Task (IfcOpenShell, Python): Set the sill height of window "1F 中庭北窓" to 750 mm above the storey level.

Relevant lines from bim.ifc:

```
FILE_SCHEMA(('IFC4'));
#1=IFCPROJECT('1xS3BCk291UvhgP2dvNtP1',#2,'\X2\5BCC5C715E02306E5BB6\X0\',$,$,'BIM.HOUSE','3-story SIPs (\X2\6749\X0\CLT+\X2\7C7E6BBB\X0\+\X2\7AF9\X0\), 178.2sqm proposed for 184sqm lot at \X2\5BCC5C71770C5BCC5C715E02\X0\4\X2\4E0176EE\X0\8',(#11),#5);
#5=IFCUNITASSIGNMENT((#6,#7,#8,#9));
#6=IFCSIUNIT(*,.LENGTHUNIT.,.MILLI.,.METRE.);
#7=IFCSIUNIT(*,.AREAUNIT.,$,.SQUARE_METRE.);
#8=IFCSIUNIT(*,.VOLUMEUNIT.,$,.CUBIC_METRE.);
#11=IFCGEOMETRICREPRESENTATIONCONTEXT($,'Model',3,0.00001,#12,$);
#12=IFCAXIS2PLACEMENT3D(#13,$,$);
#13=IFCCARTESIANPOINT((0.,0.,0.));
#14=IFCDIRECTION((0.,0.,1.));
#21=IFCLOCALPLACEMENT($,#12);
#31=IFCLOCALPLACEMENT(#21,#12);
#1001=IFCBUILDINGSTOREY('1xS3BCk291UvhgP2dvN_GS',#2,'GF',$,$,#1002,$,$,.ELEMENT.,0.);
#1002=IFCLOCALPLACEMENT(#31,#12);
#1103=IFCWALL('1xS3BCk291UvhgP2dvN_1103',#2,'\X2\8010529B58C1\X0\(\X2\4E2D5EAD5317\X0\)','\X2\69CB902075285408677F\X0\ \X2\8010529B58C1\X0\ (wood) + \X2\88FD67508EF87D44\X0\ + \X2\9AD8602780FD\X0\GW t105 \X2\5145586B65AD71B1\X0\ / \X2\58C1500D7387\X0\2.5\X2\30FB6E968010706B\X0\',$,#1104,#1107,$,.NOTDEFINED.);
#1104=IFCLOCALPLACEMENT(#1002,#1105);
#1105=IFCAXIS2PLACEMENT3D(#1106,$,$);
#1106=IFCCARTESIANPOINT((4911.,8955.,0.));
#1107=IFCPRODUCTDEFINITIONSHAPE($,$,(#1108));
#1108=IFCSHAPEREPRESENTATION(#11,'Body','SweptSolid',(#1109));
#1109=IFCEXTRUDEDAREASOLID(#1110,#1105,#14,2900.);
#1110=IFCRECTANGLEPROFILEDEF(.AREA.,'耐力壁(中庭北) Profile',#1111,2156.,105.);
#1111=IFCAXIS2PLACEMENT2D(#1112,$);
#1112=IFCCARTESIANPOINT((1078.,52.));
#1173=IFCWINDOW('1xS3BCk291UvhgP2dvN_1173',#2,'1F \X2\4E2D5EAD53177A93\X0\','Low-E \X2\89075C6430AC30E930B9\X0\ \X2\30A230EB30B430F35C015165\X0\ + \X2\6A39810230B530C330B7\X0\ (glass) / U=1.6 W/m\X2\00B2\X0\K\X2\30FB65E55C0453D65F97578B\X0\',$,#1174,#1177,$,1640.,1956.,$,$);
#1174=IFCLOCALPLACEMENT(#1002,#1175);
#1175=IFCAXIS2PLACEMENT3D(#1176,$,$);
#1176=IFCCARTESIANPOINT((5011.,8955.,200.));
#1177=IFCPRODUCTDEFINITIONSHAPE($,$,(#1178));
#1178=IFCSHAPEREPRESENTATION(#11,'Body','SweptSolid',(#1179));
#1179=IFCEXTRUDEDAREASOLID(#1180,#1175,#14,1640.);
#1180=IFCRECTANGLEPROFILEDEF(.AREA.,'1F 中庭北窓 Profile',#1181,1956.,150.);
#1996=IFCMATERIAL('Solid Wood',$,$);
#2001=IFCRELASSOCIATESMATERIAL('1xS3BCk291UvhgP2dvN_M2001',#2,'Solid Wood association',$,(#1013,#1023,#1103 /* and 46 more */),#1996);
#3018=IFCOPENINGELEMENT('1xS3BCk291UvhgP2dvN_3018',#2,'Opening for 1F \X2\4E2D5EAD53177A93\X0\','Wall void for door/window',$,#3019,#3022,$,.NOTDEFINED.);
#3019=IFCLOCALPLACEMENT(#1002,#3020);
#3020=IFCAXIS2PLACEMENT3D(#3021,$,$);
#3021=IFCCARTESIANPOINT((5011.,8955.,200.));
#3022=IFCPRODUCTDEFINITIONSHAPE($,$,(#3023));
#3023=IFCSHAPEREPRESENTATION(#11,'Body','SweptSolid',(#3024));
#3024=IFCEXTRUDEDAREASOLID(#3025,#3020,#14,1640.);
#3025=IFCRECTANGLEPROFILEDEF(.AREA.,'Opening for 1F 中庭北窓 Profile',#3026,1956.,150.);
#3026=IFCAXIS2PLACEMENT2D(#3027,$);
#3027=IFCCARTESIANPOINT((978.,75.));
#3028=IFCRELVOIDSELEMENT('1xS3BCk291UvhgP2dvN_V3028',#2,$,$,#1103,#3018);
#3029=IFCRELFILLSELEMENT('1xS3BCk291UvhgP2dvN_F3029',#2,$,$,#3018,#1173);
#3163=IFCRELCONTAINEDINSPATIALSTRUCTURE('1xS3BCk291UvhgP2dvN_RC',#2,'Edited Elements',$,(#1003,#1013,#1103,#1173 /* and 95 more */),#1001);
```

```python
import numpy as np
import ifcopenshell
import ifcopenshell.api.geometry
import ifcopenshell.geom
import ifcopenshell.util.element
import ifcopenshell.util.placement
import ifcopenshell.util.shape
import ifcopenshell.util.unit

model = ifcopenshell.open("bim.ifc")
unit_scale = ifcopenshell.util.unit.calculate_unit_scale(model)

window = model.by_guid("1xS3BCk291UvhgP2dvN_1173")
opening = window.FillsVoids[0].RelatingOpeningElement
storey = ifcopenshell.util.element.get_container(window, ifc_class="IfcBuildingStorey")
level = ifcopenshell.util.placement.get_local_placement(storey.ObjectPlacement)[2, 3]

# The opening's origin need not be at the sill, so measure its lowest point.
shape = ifcopenshell.geom.create_shape(ifcopenshell.geom.settings(), opening)
bottom = ifcopenshell.util.shape.get_shape_bottom_elevation(shape, shape.geometry) / unit_scale
dz = level + 750.0 - bottom

shift = np.array([0.0, 0.0, dz])
# The window is not placed relative to its opening, so move both.
for product in (opening, window):
    matrix = ifcopenshell.util.placement.get_local_placement(product.ObjectPlacement)
    matrix[:3, 3] += shift
    ifcopenshell.api.geometry.edit_object_placement(model, product=product, matrix=matrix, is_si=False)

print(f"moved by {dz * unit_scale:+.3f} m")

model.write("bim-out.ifc")
```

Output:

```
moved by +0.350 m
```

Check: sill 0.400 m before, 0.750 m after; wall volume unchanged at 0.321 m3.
